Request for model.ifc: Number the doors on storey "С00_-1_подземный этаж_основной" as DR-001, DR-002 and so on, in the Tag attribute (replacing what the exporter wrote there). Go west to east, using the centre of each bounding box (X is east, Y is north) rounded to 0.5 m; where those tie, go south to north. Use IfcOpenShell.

First a look at what the model holds.

```python
import ifcopenshell
import ifcopenshell.util.element
import ifcopenshell.util.placement

model = ifcopenshell.open("model.ifc")
print(model.schema)
storey = next(s for s in model.by_type("IfcBuildingStorey") if s.Name == "С00_-1_подземный этаж_основной")
doors = [e for e in ifcopenshell.util.element.get_decomposition(storey) if e.is_a("IfcDoor")]
for e in sorted(doors, key=lambda e: e.id()):
    origin = ifcopenshell.util.placement.get_local_placement(e.ObjectPlacement)[:3, 3]
    print(e.id(), e.Tag, e.Name, origin.round(2) + 0.0, sep=" | ")
```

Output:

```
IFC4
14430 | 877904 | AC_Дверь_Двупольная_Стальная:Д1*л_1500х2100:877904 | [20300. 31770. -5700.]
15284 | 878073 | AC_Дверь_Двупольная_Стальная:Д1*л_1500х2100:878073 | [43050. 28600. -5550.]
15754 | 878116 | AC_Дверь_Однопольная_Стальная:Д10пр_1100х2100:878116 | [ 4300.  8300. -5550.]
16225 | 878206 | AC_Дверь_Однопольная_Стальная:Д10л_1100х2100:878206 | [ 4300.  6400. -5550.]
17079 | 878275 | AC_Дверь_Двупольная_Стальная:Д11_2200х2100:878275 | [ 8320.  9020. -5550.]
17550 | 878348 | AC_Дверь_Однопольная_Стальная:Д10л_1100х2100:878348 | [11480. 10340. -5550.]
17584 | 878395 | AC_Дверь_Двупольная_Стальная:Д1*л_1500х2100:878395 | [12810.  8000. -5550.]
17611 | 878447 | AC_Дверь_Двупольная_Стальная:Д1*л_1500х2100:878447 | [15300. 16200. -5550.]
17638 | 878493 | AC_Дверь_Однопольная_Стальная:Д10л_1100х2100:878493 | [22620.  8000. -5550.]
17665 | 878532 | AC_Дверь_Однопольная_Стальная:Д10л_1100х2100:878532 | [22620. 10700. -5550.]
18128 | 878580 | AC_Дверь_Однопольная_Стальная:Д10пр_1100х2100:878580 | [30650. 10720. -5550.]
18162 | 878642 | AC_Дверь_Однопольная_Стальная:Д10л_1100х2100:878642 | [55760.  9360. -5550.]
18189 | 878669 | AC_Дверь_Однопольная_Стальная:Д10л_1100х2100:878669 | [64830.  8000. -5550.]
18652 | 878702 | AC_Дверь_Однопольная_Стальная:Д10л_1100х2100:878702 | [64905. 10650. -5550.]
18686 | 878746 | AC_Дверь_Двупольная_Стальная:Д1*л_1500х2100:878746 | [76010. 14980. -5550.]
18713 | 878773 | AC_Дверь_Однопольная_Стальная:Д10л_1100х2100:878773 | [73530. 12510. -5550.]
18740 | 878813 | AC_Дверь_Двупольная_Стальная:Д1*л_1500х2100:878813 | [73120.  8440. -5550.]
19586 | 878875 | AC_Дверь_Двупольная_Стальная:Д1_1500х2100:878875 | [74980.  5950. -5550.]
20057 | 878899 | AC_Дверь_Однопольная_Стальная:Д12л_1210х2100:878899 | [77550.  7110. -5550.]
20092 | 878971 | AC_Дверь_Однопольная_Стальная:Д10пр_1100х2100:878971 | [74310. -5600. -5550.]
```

```python
import ifcopenshell
import ifcopenshell.geom
import ifcopenshell.util.element
import ifcopenshell.util.shape

model = ifcopenshell.open("model.ifc")
settings = ifcopenshell.geom.settings()
settings.set("use-world-coords", True)


def centre(element):
    shape = ifcopenshell.geom.create_shape(settings, element)
    return ifcopenshell.util.shape.get_bbox_centroid(shape.geometry)


storey = next(s for s in model.by_type("IfcBuildingStorey") if s.Name == "С00_-1_подземный этаж_основной")
doors = [e for e in ifcopenshell.util.element.get_decomposition(storey) if e.is_a("IfcDoor")]

# Insertion points can sit at a corner or the storey origin, so sort by the geometry (in metres).
centres = {e: centre(e) for e in doors}
doors.sort(key=lambda e: (round(centres[e][0] / 0.5), centres[e][1]))

for i, e in enumerate(doors, start=1):
    number = f"DR-0{i:02d}"
    e.Tag = number
    print(e.id(), number)

model.write("model-out.ifc")
```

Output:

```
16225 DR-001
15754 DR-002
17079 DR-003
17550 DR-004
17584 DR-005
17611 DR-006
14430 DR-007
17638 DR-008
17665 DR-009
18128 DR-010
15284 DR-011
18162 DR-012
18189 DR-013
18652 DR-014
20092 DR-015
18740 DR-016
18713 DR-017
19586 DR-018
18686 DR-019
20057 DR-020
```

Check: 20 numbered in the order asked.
